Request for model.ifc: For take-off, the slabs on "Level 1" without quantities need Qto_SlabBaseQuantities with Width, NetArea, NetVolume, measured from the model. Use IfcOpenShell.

First a look at what the model holds.

```python
import ifcopenshell
import ifcopenshell.util.element
import ifcopenshell.util.unit

model = ifcopenshell.open("model.ifc")
print(model.schema)
for unit_type in ("LENGTHUNIT", "AREAUNIT", "VOLUMEUNIT"):
    print(unit_type, ifcopenshell.util.unit.calculate_unit_scale(model, unit_type))
storey = next(s for s in model.by_type("IfcBuildingStorey") if s.Name == "Level 1")
slabs = [e for e in ifcopenshell.util.element.get_decomposition(storey) if e.is_a("IfcSlab")]
for e in sorted(slabs, key=lambda e: e.id()):
    print(e.id(), e.is_a(), e.Name, list(ifcopenshell.util.element.get_psets(e, qtos_only=True)), sep=" | ")
```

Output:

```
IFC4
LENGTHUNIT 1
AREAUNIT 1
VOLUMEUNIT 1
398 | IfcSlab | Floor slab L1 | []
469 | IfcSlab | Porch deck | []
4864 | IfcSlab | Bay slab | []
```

```python
import ifcopenshell
import ifcopenshell.api.pset
import ifcopenshell.geom
import ifcopenshell.util.element
import ifcopenshell.util.shape
import ifcopenshell.util.unit

model = ifcopenshell.open("model.ifc")
unit_scale = ifcopenshell.util.unit.calculate_unit_scale(model)
area_scale = ifcopenshell.util.unit.calculate_unit_scale(model, "AREAUNIT")
volume_scale = ifcopenshell.util.unit.calculate_unit_scale(model, "VOLUMEUNIT")
settings = ifcopenshell.geom.settings()

storey = next(s for s in model.by_type("IfcBuildingStorey") if s.Name == "Level 1")
slabs = [e for e in ifcopenshell.util.element.get_decomposition(storey) if e.is_a("IfcSlab")]

for e in sorted(slabs, key=lambda e: e.id()):
    if ifcopenshell.util.element.get_psets(e, qtos_only=True, should_inherit=False):
        continue
    # Geometry comes back in metres, in the element's own axes.
    shape = ifcopenshell.geom.create_shape(settings, e)
    values = {
        "Width": ifcopenshell.util.shape.get_z(shape.geometry) / unit_scale,
        "NetArea": ifcopenshell.util.shape.get_footprint_area(shape.geometry) / area_scale,
        "NetVolume": ifcopenshell.util.shape.get_volume(shape.geometry) / volume_scale,
    }
    qto = ifcopenshell.api.pset.add_qto(model, product=e, name="Qto_SlabBaseQuantities")
    ifcopenshell.api.pset.edit_qto(model, qto=qto, properties=values)
    print(e.id(), {k: round(v, 3) for k, v in values.items()})

model.write("model_edited.ifc")
```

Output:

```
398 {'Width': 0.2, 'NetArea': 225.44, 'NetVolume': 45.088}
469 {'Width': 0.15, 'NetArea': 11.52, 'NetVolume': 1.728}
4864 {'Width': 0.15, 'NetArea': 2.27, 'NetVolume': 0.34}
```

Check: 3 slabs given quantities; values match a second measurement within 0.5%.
